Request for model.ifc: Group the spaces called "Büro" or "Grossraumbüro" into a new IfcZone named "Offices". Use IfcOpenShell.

First a look at what the model holds.

```python
import ifcopenshell

model = ifcopenshell.open("model.ifc")
print(model.schema)
seen = {}
for space in model.by_type("IfcSpace"):
    seen[space.LongName] = seen.get(space.LongName, 0) + 1
for name, count in sorted(seen.items(), key=str):
    print(count, "x", name)
print("zones:", [z.Name for z in model.by_type("IfcZone")][:20])
```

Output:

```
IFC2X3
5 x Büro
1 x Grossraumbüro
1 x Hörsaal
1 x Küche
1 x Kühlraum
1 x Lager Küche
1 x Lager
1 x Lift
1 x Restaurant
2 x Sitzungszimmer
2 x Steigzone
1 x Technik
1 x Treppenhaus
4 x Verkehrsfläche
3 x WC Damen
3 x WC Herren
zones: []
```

```python
import ifcopenshell
import ifcopenshell.api.group
import ifcopenshell.api.root

model = ifcopenshell.open("model.ifc")

names = {"Büro", "Grossraumbüro"}
spaces = [s for s in model.by_type("IfcSpace") if s.LongName in names]

zone = ifcopenshell.api.root.create_entity(model, ifc_class="IfcZone", name="Offices")
ifcopenshell.api.group.assign_group(model, products=spaces, group=zone)
print(len(spaces), "spaces in", zone.Name)

model.write("model_v2.ifc")
```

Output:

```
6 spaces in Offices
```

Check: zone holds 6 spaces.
